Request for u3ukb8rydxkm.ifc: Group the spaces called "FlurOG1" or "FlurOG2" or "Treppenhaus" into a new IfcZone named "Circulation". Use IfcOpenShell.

First a look at what the model holds.

```python
import ifcopenshell

model = ifcopenshell.open("u3ukb8rydxkm.ifc")
print(model.schema)
seen = {}
for space in model.by_type("IfcSpace"):
    seen[space.Name] = seen.get(space.Name, 0) + 1
for name, count in sorted(seen.items(), key=str):
    print(count, "x", name)
print("zones:", [z.Name for z in model.by_type("IfcZone")][:20])
```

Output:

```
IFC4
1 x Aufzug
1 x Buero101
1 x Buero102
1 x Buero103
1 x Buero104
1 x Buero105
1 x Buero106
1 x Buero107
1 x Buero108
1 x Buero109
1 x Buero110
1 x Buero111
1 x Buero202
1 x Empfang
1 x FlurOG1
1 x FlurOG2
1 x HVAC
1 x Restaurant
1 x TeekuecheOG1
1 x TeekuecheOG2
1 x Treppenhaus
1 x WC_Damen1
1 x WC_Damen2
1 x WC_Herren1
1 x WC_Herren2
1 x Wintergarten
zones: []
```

```python
import ifcopenshell
import ifcopenshell.api.group
import ifcopenshell.api.root

model = ifcopenshell.open("u3ukb8rydxkm.ifc")

names = {"FlurOG1", "FlurOG2", "Treppenhaus"}
spaces = [s for s in model.by_type("IfcSpace") if s.Name in names]

zone = ifcopenshell.api.root.create_entity(model, ifc_class="IfcZone", name="Circulation")
ifcopenshell.api.group.assign_group(model, products=spaces, group=zone)
print(len(spaces), "spaces in", zone.Name)

model.write("u3ukb8rydxkm_edited.ifc")
```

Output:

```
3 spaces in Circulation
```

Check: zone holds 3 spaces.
